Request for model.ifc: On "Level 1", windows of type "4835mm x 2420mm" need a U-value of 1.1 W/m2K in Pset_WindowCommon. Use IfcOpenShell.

First a look at what the model holds.

```python
import ifcopenshell
import ifcopenshell.util.element

model = ifcopenshell.open("model.ifc")
print(model.schema)
storey = next(s for s in model.by_type("IfcBuildingStorey") if s.Name == "Level 1")
windows = [e for e in ifcopenshell.util.element.get_decomposition(storey) if e.is_a("IfcWindow")]
seen = {}
for e in windows:
    element_type = ifcopenshell.util.element.get_type(e)
    key = (element_type.Name if element_type != e and element_type else None, ifcopenshell.util.element.get_pset(e, "Pset_WindowCommon", "ThermalTransmittance"))
    seen[key] = seen.get(key, 0) + 1
for (name, value), count in sorted(seen.items(), key=str):
    print(count, "x", name, "|", value)
```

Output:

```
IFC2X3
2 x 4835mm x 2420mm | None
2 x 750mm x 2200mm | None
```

```python
import ifcopenshell
import ifcopenshell.api.pset
import ifcopenshell.util.element

model = ifcopenshell.open("model.ifc")

storey = next(s for s in model.by_type("IfcBuildingStorey") if s.Name == "Level 1")
windows = [e for e in ifcopenshell.util.element.get_decomposition(storey) if e.is_a("IfcWindow")]

count = 0
for e in windows:
    element_type = ifcopenshell.util.element.get_type(e)
    if element_type in (None, e) or element_type.Name != "4835mm x 2420mm":
        continue
    # add_pset returns the element's existing set when there is one.
    pset = ifcopenshell.api.pset.add_pset(model, product=e, name="Pset_WindowCommon")
    ifcopenshell.api.pset.edit_pset(model, pset=pset, properties={"ThermalTransmittance": 1.1})
    count += 1

print(count, "windows updated")

model.write("model_edited.ifc")
```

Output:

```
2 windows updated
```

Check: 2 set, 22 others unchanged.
